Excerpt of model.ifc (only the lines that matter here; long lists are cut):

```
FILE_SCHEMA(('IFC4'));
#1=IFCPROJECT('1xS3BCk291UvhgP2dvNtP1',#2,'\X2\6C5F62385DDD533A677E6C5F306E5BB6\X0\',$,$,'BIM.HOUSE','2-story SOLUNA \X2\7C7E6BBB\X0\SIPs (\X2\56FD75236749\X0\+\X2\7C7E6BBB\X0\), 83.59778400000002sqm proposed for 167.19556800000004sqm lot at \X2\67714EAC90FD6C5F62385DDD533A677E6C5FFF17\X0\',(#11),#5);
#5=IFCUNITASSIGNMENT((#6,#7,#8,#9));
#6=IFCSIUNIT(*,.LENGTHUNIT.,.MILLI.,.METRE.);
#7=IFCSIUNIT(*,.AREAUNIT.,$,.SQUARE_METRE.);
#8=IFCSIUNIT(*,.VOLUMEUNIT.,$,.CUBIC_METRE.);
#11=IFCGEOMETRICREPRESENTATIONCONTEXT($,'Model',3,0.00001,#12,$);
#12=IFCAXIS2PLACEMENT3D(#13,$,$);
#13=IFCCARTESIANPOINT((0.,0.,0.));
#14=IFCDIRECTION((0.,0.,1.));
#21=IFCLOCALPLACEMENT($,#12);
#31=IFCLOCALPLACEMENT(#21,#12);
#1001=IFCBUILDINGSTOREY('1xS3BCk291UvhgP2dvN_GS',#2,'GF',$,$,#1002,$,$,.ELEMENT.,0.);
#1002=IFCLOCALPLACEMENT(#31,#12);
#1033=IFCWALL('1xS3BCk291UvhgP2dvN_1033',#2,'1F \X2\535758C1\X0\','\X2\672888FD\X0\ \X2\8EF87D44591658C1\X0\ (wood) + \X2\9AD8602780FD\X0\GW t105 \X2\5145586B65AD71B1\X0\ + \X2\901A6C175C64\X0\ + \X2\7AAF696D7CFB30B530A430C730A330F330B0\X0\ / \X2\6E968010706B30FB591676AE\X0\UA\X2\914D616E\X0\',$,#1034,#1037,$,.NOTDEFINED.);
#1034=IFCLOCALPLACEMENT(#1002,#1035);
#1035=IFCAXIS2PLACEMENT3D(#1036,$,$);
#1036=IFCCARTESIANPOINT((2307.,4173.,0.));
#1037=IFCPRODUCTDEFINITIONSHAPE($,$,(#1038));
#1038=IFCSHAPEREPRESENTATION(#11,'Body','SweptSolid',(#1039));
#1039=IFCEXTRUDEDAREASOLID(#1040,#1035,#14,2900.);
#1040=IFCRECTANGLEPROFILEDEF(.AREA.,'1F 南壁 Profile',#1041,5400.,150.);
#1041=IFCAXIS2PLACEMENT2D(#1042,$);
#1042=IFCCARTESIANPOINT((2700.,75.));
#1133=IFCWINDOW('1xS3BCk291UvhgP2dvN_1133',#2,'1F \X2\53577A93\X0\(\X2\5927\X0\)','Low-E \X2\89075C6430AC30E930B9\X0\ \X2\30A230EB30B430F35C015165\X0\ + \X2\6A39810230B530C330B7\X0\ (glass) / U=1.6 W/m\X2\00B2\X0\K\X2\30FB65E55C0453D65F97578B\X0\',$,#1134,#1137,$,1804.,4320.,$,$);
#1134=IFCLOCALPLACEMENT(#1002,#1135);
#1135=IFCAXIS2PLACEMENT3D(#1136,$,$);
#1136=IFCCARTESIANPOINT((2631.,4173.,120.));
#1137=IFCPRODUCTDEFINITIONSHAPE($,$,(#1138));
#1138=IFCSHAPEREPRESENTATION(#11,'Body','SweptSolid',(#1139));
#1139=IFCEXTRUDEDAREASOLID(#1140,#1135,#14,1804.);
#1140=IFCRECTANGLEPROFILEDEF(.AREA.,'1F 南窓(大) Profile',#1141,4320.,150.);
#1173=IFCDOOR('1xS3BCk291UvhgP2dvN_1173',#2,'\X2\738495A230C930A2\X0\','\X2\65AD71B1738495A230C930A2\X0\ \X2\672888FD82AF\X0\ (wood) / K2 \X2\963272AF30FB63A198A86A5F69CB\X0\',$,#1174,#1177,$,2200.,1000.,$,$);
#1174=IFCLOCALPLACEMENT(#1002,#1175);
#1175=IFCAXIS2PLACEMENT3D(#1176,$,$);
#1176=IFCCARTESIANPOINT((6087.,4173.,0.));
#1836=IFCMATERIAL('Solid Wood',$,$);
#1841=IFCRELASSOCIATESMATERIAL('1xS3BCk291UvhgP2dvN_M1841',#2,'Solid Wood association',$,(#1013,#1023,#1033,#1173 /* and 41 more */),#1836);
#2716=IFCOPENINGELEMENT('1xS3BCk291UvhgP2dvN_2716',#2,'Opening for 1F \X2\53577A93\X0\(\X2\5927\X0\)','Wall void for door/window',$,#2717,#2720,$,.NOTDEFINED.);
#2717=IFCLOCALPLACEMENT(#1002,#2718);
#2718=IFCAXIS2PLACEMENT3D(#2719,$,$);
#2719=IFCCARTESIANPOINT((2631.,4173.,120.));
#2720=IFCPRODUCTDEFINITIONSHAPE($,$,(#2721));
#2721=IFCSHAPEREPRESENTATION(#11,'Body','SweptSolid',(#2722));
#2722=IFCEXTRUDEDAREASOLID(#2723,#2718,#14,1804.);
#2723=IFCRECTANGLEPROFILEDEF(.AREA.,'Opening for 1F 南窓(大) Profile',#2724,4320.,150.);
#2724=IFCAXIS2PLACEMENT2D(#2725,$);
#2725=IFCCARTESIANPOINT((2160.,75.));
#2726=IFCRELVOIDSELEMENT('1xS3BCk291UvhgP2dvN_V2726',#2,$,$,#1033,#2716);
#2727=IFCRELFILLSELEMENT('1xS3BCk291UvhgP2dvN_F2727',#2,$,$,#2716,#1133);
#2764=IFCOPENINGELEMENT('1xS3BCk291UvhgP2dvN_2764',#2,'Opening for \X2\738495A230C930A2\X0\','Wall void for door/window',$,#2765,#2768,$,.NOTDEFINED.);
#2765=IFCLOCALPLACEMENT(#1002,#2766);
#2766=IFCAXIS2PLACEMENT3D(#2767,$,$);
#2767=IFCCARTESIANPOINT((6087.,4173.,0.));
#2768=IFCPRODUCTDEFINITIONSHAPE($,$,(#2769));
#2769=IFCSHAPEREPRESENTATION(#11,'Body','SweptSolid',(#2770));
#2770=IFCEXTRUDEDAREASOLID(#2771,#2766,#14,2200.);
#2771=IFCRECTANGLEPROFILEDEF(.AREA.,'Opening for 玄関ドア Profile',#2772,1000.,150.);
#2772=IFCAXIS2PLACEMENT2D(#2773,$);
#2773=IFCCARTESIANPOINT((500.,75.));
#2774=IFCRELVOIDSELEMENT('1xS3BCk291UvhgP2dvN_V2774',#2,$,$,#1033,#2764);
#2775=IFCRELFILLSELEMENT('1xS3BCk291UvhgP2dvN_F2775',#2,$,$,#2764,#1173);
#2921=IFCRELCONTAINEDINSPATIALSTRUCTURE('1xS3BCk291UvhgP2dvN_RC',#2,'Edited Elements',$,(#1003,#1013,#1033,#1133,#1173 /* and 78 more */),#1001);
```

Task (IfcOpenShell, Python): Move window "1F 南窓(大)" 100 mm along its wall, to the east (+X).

```python
import ifcopenshell
import ifcopenshell.api.geometry
import ifcopenshell.util.placement
import ifcopenshell.util.unit

model = ifcopenshell.open("model.ifc")
unit_scale = ifcopenshell.util.unit.calculate_unit_scale(model)

window = model.by_id(1133)
opening = window.FillsVoids[0].RelatingOpeningElement
wall = opening.VoidsElements[0].RelatingBuildingElement

wall_matrix = ifcopenshell.util.placement.get_local_placement(wall.ObjectPlacement)
shift = wall_matrix[:3, 0] * 0.1 / unit_scale
before = ifcopenshell.util.placement.get_local_placement(window.ObjectPlacement)[:3, 3].copy()

# The window is not placed relative to its opening, so move both.
for product in (opening, window):
    matrix = ifcopenshell.util.placement.get_local_placement(product.ObjectPlacement)
    matrix[:3, 3] += shift
    ifcopenshell.api.geometry.edit_object_placement(model, product=product, matrix=matrix, is_si=False)

after = ifcopenshell.util.placement.get_local_placement(window.ObjectPlacement)[:3, 3]
print("window moved by", (after - before).round(3) + 0.0)

model.write("model_rev.ifc")
```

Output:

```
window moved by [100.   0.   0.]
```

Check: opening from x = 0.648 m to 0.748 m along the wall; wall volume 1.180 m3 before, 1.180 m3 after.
